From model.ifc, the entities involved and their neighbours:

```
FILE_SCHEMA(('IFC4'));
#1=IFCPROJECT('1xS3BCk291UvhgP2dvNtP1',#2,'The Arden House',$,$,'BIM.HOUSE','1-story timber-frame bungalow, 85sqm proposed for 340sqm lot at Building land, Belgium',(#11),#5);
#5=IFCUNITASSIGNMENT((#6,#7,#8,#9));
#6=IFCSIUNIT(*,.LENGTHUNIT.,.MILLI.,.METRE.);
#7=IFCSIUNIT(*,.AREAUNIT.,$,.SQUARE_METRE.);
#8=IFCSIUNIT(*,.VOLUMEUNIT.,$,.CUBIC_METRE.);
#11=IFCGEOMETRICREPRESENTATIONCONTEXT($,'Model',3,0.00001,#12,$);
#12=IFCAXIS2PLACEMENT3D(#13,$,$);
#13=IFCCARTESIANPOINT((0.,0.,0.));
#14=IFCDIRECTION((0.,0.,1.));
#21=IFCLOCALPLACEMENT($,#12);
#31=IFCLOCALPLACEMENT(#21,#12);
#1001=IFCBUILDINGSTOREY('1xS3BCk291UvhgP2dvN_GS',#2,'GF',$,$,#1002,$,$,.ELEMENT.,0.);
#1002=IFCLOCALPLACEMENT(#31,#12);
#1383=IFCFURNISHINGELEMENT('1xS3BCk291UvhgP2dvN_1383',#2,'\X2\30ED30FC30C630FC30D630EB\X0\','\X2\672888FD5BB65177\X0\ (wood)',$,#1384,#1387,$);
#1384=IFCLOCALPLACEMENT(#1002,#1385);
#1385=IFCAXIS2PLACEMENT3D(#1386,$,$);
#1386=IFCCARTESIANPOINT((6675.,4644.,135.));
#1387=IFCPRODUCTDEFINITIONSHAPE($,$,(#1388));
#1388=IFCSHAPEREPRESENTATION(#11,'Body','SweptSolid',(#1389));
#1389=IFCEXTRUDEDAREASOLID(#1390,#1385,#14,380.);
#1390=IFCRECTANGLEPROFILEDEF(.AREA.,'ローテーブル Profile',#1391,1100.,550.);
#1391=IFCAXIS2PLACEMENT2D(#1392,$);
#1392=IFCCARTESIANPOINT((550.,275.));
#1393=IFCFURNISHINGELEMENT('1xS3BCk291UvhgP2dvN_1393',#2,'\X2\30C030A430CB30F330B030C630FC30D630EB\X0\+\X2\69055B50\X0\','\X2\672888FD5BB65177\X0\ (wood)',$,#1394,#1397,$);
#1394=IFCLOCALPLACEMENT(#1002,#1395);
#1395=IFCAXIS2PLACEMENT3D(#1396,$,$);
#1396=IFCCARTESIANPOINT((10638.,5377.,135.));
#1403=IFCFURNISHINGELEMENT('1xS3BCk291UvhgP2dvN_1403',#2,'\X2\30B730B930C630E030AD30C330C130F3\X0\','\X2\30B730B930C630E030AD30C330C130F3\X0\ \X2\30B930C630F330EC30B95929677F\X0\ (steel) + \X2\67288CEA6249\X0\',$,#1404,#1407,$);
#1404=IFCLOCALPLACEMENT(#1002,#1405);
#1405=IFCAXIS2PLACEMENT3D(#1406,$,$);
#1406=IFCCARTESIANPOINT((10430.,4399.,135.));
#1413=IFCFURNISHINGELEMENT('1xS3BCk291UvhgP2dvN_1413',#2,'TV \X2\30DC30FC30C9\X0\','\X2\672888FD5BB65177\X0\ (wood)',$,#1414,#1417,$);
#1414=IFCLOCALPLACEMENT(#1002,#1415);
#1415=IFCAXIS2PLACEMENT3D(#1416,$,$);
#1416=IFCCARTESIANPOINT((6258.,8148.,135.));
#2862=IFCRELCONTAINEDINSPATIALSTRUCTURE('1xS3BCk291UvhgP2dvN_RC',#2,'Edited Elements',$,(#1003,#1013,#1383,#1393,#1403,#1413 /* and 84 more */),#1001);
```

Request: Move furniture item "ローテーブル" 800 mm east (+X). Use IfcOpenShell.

```python
import ifcopenshell
import ifcopenshell.api.geometry
import ifcopenshell.util.placement

model = ifcopenshell.open("model.ifc")

item = model.by_id(1383)
matrix = ifcopenshell.util.placement.get_local_placement(item.ObjectPlacement)
matrix[0, 3] += 800.0
ifcopenshell.api.geometry.edit_object_placement(model, product=item, matrix=matrix, is_si=False)

print(ifcopenshell.util.placement.get_local_placement(item.ObjectPlacement).round(3) + 0.0)

model.write("model_rev.ifc")
```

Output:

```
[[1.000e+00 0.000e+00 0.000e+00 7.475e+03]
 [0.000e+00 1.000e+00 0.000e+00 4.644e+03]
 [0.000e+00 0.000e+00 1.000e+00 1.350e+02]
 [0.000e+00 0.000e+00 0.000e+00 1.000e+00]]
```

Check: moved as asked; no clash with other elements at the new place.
